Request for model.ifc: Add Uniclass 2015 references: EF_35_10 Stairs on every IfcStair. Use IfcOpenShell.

First a look at what the model holds.

```python
import ifcopenshell

model = ifcopenshell.open("model.ifc")
print(model.schema)
print("classifications:", [c.Name for c in model.by_type("IfcClassification")])
for ifc_class in ("IfcDoor", "IfcRoof", "IfcStair", "IfcWall", "IfcWindow"):
    print(ifc_class, len(model.by_type(ifc_class)))
```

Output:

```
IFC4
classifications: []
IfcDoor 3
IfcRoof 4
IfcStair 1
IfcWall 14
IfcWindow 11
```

```python
import ifcopenshell
import ifcopenshell.api.classification

model = ifcopenshell.open("model.ifc")

system = ifcopenshell.api.classification.add_classification(model, classification="Uniclass 2015")

codes = {
    "IfcStair": ("EF_35_10", "Stairs"),
}
for ifc_class, (code, name) in codes.items():
    products = model.by_type(ifc_class)
    ifcopenshell.api.classification.add_reference(
        model, products=products, classification=system, identification=code, name=name
    )
    print(code, len(products))

model.write("model_updated.ifc")
```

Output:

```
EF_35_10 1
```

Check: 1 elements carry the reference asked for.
